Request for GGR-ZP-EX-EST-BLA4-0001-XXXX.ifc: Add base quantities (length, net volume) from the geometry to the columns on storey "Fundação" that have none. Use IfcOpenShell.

First a look at what the model holds.

```python
import ifcopenshell
import ifcopenshell.util.element
import ifcopenshell.util.unit

model = ifcopenshell.open("GGR-ZP-EX-EST-BLA4-0001-XXXX.ifc")
print(model.schema)
for unit_type in ("LENGTHUNIT", "AREAUNIT", "VOLUMEUNIT"):
    print(unit_type, ifcopenshell.util.unit.calculate_unit_scale(model, unit_type))
storey = next(s for s in model.by_type("IfcBuildingStorey") if s.Name == "Fundação")
columns = [e for e in ifcopenshell.util.element.get_decomposition(storey) if e.is_a("IfcColumn")]
for e in sorted(columns, key=lambda e: e.id()):
    print(e.id(), e.is_a(), e.Name, list(ifcopenshell.util.element.get_psets(e, qtos_only=True)), sep=" | ")
```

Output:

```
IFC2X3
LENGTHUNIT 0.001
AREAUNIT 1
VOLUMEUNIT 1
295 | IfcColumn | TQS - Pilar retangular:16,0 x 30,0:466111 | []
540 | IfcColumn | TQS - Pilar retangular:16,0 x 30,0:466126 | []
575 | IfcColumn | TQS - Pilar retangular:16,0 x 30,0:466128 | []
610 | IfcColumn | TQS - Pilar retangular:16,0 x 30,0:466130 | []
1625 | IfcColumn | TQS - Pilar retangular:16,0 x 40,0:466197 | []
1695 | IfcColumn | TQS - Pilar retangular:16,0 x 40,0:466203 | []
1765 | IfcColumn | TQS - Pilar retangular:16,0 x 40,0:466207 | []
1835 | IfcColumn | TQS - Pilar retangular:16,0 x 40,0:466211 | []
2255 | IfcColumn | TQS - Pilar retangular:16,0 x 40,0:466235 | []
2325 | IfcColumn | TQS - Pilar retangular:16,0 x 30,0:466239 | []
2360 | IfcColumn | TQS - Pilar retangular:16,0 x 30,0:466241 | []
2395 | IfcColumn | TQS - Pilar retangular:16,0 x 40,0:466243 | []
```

```python
import ifcopenshell
import ifcopenshell.api.pset
import ifcopenshell.geom
import ifcopenshell.util.element
import ifcopenshell.util.shape
import ifcopenshell.util.unit

model = ifcopenshell.open("GGR-ZP-EX-EST-BLA4-0001-XXXX.ifc")
unit_scale = ifcopenshell.util.unit.calculate_unit_scale(model)
volume_scale = ifcopenshell.util.unit.calculate_unit_scale(model, "VOLUMEUNIT")
settings = ifcopenshell.geom.settings()

storey = next(s for s in model.by_type("IfcBuildingStorey") if s.Name == "Fundação")
columns = [e for e in ifcopenshell.util.element.get_decomposition(storey) if e.is_a("IfcColumn")]

for e in sorted(columns, key=lambda e: e.id()):
    if ifcopenshell.util.element.get_psets(e, qtos_only=True, should_inherit=False):
        continue
    # Geometry comes back in metres, in the element's own axes.
    shape = ifcopenshell.geom.create_shape(settings, e)
    values = {
        "Length": ifcopenshell.util.shape.get_z(shape.geometry) / unit_scale,
        "NetVolume": ifcopenshell.util.shape.get_volume(shape.geometry) / volume_scale,
    }
    qto = ifcopenshell.api.pset.add_qto(model, product=e, name="BaseQuantities")
    ifcopenshell.api.pset.edit_qto(model, qto=qto, properties=values)
    print(e.id(), {k: round(v, 3) for k, v in values.items()})

model.write("GGR-ZP-EX-EST-BLA4-0001-XXXX_v2.ifc")
```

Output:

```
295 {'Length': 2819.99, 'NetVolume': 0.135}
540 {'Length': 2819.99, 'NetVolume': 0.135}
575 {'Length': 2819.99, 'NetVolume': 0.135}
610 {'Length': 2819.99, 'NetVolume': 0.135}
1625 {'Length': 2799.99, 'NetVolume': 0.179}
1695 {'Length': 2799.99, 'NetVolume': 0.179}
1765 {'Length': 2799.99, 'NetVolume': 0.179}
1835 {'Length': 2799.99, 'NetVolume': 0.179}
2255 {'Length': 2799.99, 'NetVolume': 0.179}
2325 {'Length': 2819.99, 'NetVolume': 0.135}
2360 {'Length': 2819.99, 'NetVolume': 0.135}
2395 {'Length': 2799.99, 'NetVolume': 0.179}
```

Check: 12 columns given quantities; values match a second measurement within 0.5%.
